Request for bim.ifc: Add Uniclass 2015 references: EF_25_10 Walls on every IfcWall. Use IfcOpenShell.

First a look at what the model holds.

```python
import ifcopenshell

model = ifcopenshell.open("bim.ifc")
print(model.schema)
print("classifications:", [c.Name for c in model.by_type("IfcClassification")])
for ifc_class in ("IfcDoor", "IfcRoof", "IfcStair", "IfcWall", "IfcWindow"):
    print(ifc_class, len(model.by_type(ifc_class)))
```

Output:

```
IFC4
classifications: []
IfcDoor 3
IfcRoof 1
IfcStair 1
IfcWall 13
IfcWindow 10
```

```python
import ifcopenshell
import ifcopenshell.api.classification

model = ifcopenshell.open("bim.ifc")

system = ifcopenshell.api.classification.add_classification(model, classification="Uniclass 2015")

codes = {
    "IfcWall": ("EF_25_10", "Walls"),
}
for ifc_class, (code, name) in codes.items():
    products = model.by_type(ifc_class)
    ifcopenshell.api.classification.add_reference(
        model, products=products, classification=system, identification=code, name=name
    )
    print(code, len(products))

model.write("bim_updated.ifc")
```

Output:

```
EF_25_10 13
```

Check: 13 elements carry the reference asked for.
